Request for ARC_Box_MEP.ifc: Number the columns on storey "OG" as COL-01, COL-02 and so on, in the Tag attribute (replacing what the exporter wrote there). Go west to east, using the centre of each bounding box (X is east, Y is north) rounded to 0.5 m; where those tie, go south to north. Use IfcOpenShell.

First a look at what the model holds.

```python
import ifcopenshell
import ifcopenshell.util.element
import ifcopenshell.util.placement

model = ifcopenshell.open("ARC_Box_MEP.ifc")
print(model.schema)
storey = next(s for s in model.by_type("IfcBuildingStorey") if s.Name == "OG")
columns = [e for e in ifcopenshell.util.element.get_decomposition(storey) if e.is_a("IfcColumn")]
for e in sorted(columns, key=lambda e: e.id()):
    origin = ifcopenshell.util.placement.get_local_placement(e.ObjectPlacement)[:3, 3]
    print(e.id(), e.Tag, e.Name, origin.round(2) + 0.0, sep=" | ")
```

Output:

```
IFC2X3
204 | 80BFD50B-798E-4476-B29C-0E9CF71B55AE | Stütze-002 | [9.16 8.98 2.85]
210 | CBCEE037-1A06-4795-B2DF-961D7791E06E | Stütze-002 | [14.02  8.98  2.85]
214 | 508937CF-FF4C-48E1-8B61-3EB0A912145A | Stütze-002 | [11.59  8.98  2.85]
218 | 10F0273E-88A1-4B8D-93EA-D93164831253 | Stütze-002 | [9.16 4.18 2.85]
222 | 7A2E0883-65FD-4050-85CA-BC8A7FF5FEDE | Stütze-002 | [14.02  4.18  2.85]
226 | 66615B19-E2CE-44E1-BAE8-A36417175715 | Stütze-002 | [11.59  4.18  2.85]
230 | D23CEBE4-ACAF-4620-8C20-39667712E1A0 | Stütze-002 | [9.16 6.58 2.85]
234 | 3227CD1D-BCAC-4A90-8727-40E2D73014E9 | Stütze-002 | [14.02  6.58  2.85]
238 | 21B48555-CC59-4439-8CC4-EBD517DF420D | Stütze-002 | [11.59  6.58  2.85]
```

```python
import ifcopenshell
import ifcopenshell.geom
import ifcopenshell.util.element
import ifcopenshell.util.shape

model = ifcopenshell.open("ARC_Box_MEP.ifc")
settings = ifcopenshell.geom.settings()
settings.set("use-world-coords", True)


def centre(element):
    shape = ifcopenshell.geom.create_shape(settings, element)
    return ifcopenshell.util.shape.get_bbox_centroid(shape.geometry)


storey = next(s for s in model.by_type("IfcBuildingStorey") if s.Name == "OG")
columns = [e for e in ifcopenshell.util.element.get_decomposition(storey) if e.is_a("IfcColumn")]

# Insertion points can sit at a corner or the storey origin, so sort by the geometry (in metres).
centres = {e: centre(e) for e in columns}
columns.sort(key=lambda e: (round(centres[e][0] / 0.5), centres[e][1]))

for i, e in enumerate(columns, start=1):
    number = f"COL-{i:02d}"
    e.Tag = number
    print(e.id(), number)

model.write("ARC_Box_MEP-out.ifc")
```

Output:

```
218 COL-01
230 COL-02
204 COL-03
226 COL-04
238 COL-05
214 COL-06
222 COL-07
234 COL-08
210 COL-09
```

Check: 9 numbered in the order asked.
